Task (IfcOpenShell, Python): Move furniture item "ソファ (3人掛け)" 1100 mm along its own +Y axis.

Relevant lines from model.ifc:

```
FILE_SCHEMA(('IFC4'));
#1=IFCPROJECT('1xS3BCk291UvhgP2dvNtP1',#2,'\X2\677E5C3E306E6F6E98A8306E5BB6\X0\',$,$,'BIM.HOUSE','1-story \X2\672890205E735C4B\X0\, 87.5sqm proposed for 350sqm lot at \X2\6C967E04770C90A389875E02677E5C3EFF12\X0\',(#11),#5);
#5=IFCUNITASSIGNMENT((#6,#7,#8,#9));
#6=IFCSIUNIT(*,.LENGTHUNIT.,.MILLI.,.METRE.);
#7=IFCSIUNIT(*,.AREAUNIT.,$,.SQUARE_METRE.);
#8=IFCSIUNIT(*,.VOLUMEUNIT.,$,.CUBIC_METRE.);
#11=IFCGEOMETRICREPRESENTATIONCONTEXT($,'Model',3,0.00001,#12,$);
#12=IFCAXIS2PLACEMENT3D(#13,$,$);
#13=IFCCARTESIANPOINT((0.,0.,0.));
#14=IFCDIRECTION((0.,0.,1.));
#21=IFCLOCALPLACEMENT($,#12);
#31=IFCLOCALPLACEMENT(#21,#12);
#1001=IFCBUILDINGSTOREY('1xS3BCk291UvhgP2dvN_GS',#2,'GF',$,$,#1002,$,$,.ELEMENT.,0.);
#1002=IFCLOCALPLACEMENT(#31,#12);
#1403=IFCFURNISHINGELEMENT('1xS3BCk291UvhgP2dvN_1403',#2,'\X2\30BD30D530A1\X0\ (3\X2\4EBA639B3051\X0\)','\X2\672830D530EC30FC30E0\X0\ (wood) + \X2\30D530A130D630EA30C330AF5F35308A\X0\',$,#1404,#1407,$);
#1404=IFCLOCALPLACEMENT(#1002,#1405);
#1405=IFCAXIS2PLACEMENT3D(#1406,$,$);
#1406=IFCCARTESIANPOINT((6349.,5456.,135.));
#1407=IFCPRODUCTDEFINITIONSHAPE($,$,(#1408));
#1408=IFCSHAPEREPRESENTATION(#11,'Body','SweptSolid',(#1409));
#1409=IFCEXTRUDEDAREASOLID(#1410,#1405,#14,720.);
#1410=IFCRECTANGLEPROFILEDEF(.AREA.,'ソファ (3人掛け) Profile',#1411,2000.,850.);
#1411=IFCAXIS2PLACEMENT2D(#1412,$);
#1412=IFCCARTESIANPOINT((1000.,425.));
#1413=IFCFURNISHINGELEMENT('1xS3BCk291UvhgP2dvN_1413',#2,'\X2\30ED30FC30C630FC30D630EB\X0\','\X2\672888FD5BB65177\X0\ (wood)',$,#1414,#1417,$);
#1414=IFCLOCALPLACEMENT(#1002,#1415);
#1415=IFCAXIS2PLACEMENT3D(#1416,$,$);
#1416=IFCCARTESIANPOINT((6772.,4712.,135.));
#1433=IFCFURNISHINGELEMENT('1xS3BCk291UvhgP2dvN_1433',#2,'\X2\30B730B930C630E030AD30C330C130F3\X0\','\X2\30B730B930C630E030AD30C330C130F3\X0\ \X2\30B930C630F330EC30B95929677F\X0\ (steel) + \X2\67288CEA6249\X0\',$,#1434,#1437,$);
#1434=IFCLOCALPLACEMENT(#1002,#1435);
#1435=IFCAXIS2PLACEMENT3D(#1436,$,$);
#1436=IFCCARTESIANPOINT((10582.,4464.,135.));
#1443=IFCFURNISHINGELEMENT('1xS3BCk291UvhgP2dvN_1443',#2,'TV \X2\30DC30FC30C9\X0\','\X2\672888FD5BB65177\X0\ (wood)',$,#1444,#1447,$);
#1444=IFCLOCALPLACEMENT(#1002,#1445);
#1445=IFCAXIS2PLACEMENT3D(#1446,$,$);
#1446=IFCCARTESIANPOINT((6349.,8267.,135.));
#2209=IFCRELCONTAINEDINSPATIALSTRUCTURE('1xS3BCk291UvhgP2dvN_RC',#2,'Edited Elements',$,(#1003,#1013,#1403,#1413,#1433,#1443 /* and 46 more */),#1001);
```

```python
import ifcopenshell
import ifcopenshell.api.geometry
import ifcopenshell.util.placement
import ifcopenshell.util.unit

model = ifcopenshell.open("model.ifc")
unit_scale = ifcopenshell.util.unit.calculate_unit_scale(model)

item = model.by_id(1403)
matrix = ifcopenshell.util.placement.get_local_placement(item.ObjectPlacement)
matrix[:3, 3] += matrix[:3, 1] * 1.1 / unit_scale
ifcopenshell.api.geometry.edit_object_placement(model, product=item, matrix=matrix, is_si=False)

print(ifcopenshell.util.placement.get_local_placement(item.ObjectPlacement).round(3) + 0.0)

model.write("model_v2.ifc")
```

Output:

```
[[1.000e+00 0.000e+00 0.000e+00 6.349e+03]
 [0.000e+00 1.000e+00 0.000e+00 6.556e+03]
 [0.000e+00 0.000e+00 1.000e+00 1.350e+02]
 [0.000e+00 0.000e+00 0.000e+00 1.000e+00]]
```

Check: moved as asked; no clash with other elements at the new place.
